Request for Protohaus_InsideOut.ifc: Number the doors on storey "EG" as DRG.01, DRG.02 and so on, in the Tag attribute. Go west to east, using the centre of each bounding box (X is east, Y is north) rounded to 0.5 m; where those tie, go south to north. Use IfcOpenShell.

First a look at what the model holds.

```python
import ifcopenshell
import ifcopenshell.util.element
import ifcopenshell.util.placement

model = ifcopenshell.open("Protohaus_InsideOut.ifc")
print(model.schema)
storey = next(s for s in model.by_type("IfcBuildingStorey") if s.Name == "EG")
doors = [e for e in ifcopenshell.util.element.get_decomposition(storey) if e.is_a("IfcDoor")]
for e in sorted(doors, key=lambda e: e.id()):
    origin = ifcopenshell.util.placement.get_local_placement(e.ObjectPlacement)[:3, 3]
    print(e.id(), e.Tag, e.Name, origin.round(2) + 0.0, sep=" | ")
```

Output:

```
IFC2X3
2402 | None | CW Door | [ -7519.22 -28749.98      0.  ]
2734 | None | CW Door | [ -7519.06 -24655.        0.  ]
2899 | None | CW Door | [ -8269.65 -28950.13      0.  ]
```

```python
import ifcopenshell
import ifcopenshell.geom
import ifcopenshell.util.element
import ifcopenshell.util.shape

model = ifcopenshell.open("Protohaus_InsideOut.ifc")
settings = ifcopenshell.geom.settings()
settings.set("use-world-coords", True)


def centre(element):
    shape = ifcopenshell.geom.create_shape(settings, element)
    return ifcopenshell.util.shape.get_bbox_centroid(shape.geometry)


storey = next(s for s in model.by_type("IfcBuildingStorey") if s.Name == "EG")
doors = [e for e in ifcopenshell.util.element.get_decomposition(storey) if e.is_a("IfcDoor")]

# Insertion points can sit at a corner or the storey origin, so sort by the geometry (in metres).
centres = {e: centre(e) for e in doors}
doors.sort(key=lambda e: (round(centres[e][0] / 0.5), centres[e][1]))

for i, e in enumerate(doors, start=1):
    number = f"DRG.{i:02d}"
    e.Tag = number
    print(e.id(), number)

model.write("Protohaus_InsideOut_rev.ifc")
```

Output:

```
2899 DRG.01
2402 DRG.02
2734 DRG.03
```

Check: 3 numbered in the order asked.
